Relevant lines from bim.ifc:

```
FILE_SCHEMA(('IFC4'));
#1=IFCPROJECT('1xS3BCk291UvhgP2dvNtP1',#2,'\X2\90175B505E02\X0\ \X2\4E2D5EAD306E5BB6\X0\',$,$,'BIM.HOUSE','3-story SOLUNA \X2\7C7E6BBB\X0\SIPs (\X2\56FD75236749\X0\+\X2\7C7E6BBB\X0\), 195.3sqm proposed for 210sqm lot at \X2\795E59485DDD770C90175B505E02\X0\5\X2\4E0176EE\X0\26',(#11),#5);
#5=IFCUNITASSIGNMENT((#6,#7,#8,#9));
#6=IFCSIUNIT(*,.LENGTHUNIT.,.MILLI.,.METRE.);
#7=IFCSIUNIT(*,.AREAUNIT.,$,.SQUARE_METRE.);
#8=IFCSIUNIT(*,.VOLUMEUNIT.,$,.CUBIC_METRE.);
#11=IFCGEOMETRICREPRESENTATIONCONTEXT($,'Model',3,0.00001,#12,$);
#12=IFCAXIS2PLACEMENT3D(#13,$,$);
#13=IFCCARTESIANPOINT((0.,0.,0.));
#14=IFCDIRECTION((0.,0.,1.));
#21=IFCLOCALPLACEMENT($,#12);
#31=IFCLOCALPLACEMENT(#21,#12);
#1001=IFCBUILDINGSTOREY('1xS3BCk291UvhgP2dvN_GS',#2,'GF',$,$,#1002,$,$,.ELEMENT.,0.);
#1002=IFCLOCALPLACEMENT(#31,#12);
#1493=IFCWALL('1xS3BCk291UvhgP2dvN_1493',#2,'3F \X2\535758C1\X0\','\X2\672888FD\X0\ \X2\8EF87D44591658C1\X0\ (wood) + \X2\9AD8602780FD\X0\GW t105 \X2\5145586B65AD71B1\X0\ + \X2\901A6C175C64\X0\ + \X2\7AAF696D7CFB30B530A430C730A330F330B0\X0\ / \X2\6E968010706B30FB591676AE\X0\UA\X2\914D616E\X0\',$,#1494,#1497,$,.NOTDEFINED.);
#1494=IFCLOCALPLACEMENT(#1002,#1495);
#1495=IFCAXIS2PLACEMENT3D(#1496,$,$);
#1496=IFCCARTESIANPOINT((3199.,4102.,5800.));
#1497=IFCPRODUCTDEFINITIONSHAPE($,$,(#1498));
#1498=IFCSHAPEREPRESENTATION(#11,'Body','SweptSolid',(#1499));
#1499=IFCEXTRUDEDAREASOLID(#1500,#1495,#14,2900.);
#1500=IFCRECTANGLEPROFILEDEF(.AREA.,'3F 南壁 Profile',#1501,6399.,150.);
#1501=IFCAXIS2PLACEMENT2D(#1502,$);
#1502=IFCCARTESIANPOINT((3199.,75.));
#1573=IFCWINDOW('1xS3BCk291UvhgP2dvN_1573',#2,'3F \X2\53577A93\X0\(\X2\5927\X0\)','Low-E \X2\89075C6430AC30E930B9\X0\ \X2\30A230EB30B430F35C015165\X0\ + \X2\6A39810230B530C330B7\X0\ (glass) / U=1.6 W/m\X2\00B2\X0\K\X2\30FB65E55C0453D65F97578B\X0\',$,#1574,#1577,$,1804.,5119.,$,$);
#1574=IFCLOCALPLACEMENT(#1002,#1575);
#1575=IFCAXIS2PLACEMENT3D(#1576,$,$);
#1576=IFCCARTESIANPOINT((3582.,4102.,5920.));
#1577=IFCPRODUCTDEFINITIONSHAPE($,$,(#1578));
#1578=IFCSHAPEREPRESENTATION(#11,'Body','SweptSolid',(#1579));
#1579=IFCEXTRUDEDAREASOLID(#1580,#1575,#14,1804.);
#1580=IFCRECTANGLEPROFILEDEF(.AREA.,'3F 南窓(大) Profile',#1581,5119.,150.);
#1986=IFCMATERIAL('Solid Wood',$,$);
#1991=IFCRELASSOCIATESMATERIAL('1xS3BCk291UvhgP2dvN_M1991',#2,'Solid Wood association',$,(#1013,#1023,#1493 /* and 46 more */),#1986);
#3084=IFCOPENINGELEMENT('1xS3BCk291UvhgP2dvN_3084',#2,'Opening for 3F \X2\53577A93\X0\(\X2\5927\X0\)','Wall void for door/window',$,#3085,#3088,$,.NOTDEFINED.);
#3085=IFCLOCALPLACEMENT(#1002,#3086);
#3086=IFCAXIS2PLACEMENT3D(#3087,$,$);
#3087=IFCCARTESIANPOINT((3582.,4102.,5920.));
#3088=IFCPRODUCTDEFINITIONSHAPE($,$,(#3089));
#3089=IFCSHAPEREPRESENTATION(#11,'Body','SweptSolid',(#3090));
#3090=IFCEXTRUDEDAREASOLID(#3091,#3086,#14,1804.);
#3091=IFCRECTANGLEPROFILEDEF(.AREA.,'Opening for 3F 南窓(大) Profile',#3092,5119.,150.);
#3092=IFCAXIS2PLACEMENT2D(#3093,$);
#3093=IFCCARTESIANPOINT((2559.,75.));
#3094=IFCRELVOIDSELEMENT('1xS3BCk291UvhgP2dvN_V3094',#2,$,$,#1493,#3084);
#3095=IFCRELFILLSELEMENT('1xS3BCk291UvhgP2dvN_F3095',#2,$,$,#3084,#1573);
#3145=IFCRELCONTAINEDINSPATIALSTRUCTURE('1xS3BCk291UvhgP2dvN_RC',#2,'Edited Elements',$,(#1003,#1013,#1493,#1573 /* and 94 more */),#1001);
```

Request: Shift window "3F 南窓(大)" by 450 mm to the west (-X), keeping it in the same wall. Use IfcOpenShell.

```python
import ifcopenshell
import ifcopenshell.api.geometry
import ifcopenshell.util.placement
import ifcopenshell.util.unit

model = ifcopenshell.open("bim.ifc")
unit_scale = ifcopenshell.util.unit.calculate_unit_scale(model)

window = model.by_guid("1xS3BCk291UvhgP2dvN_1573")
opening = window.FillsVoids[0].RelatingOpeningElement
wall = opening.VoidsElements[0].RelatingBuildingElement

wall_matrix = ifcopenshell.util.placement.get_local_placement(wall.ObjectPlacement)
shift = wall_matrix[:3, 0] * -0.45 / unit_scale
before = ifcopenshell.util.placement.get_local_placement(window.ObjectPlacement)[:3, 3].copy()

# The window is not placed relative to its opening, so move both.
for product in (opening, window):
    matrix = ifcopenshell.util.placement.get_local_placement(product.ObjectPlacement)
    matrix[:3, 3] += shift
    ifcopenshell.api.geometry.edit_object_placement(model, product=product, matrix=matrix, is_si=False)

after = ifcopenshell.util.placement.get_local_placement(window.ObjectPlacement)[:3, 3]
print("window moved by", (after - before).round(3) + 0.0)

model.write("bim_edited.ifc")
```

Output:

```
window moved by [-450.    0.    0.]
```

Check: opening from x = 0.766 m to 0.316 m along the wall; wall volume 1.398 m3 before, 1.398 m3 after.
